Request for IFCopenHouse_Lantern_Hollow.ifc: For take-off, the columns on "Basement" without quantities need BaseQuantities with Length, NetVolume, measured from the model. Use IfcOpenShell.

First a look at what the model holds.

```python
import ifcopenshell
import ifcopenshell.util.element
import ifcopenshell.util.unit

model = ifcopenshell.open("IFCopenHouse_Lantern_Hollow.ifc")
print(model.schema)
for unit_type in ("LENGTHUNIT", "AREAUNIT", "VOLUMEUNIT"):
    print(unit_type, ifcopenshell.util.unit.calculate_unit_scale(model, unit_type))
storey = next(s for s in model.by_type("IfcBuildingStorey") if s.Name == "Basement")
columns = [e for e in ifcopenshell.util.element.get_decomposition(storey) if e.is_a("IfcColumn")]
for e in sorted(columns, key=lambda e: e.id()):
    print(e.id(), e.is_a(), e.Name, list(ifcopenshell.util.element.get_psets(e, qtos_only=True)), sep=" | ")
```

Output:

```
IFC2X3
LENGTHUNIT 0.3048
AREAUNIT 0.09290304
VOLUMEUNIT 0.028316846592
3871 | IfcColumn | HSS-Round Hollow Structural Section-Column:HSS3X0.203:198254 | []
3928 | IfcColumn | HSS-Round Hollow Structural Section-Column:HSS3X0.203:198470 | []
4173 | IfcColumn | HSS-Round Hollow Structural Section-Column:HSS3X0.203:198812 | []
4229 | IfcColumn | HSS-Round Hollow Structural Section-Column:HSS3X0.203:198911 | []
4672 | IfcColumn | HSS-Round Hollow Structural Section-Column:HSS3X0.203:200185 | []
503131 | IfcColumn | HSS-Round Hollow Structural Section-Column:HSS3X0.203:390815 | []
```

```python
import ifcopenshell
import ifcopenshell.api.pset
import ifcopenshell.geom
import ifcopenshell.util.element
import ifcopenshell.util.shape
import ifcopenshell.util.unit

model = ifcopenshell.open("IFCopenHouse_Lantern_Hollow.ifc")
unit_scale = ifcopenshell.util.unit.calculate_unit_scale(model)
volume_scale = ifcopenshell.util.unit.calculate_unit_scale(model, "VOLUMEUNIT")
settings = ifcopenshell.geom.settings()

storey = next(s for s in model.by_type("IfcBuildingStorey") if s.Name == "Basement")
columns = [e for e in ifcopenshell.util.element.get_decomposition(storey) if e.is_a("IfcColumn")]

for e in sorted(columns, key=lambda e: e.id()):
    if ifcopenshell.util.element.get_psets(e, qtos_only=True, should_inherit=False):
        continue
    # Geometry comes back in metres, in the element's own axes.
    shape = ifcopenshell.geom.create_shape(settings, e)
    values = {
        "Length": ifcopenshell.util.shape.get_z(shape.geometry) / unit_scale,
        "NetVolume": ifcopenshell.util.shape.get_volume(shape.geometry) / volume_scale,
    }
    qto = ifcopenshell.api.pset.add_qto(model, product=e, name="BaseQuantities")
    ifcopenshell.api.pset.edit_qto(model, qto=qto, properties=values)
    print(e.id(), {k: round(v, 3) for k, v in values.items()})

model.write("IFCopenHouse_Lantern_Hollow_updated.ifc")
```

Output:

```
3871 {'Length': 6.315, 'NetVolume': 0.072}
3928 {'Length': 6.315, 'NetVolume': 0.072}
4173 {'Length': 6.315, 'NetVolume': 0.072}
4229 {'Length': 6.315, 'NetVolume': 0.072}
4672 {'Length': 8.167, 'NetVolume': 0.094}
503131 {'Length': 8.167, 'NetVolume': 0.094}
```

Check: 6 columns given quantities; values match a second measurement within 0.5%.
